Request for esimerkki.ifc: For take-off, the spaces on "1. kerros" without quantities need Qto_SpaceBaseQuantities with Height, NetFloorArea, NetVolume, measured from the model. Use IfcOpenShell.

First a look at what the model holds.

```python
import ifcopenshell
import ifcopenshell.util.element
import ifcopenshell.util.unit

model = ifcopenshell.open("esimerkki.ifc")
print(model.schema)
for unit_type in ("LENGTHUNIT", "AREAUNIT", "VOLUMEUNIT"):
    print(unit_type, ifcopenshell.util.unit.calculate_unit_scale(model, unit_type))
storey = next(s for s in model.by_type("IfcBuildingStorey") if s.Name == "1. kerros")
spaces = [e for e in ifcopenshell.util.element.get_decomposition(storey) if e.is_a("IfcSpace")]
for e in sorted(spaces, key=lambda e: e.id()):
    print(e.id(), e.is_a(), e.Name, list(ifcopenshell.util.element.get_psets(e, qtos_only=True)), sep=" | ")
```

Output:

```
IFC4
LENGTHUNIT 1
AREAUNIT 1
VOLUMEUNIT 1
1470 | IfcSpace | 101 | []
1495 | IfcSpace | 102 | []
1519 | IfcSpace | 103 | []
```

```python
import ifcopenshell
import ifcopenshell.api.pset
import ifcopenshell.geom
import ifcopenshell.util.element
import ifcopenshell.util.shape
import ifcopenshell.util.unit

model = ifcopenshell.open("esimerkki.ifc")
unit_scale = ifcopenshell.util.unit.calculate_unit_scale(model)
area_scale = ifcopenshell.util.unit.calculate_unit_scale(model, "AREAUNIT")
volume_scale = ifcopenshell.util.unit.calculate_unit_scale(model, "VOLUMEUNIT")
settings = ifcopenshell.geom.settings()

storey = next(s for s in model.by_type("IfcBuildingStorey") if s.Name == "1. kerros")
spaces = [e for e in ifcopenshell.util.element.get_decomposition(storey) if e.is_a("IfcSpace")]

for e in sorted(spaces, key=lambda e: e.id()):
    if ifcopenshell.util.element.get_psets(e, qtos_only=True, should_inherit=False):
        continue
    # Geometry comes back in metres, in the element's own axes.
    shape = ifcopenshell.geom.create_shape(settings, e)
    values = {
        "Height": ifcopenshell.util.shape.get_z(shape.geometry) / unit_scale,
        "NetFloorArea": ifcopenshell.util.shape.get_footprint_area(shape.geometry) / area_scale,
        "NetVolume": ifcopenshell.util.shape.get_volume(shape.geometry) / volume_scale,
    }
    qto = ifcopenshell.api.pset.add_qto(model, product=e, name="Qto_SpaceBaseQuantities")
    ifcopenshell.api.pset.edit_qto(model, qto=qto, properties=values)
    print(e.id(), {k: round(v, 3) for k, v in values.items()})

model.write("esimerkki_v2.ifc")
```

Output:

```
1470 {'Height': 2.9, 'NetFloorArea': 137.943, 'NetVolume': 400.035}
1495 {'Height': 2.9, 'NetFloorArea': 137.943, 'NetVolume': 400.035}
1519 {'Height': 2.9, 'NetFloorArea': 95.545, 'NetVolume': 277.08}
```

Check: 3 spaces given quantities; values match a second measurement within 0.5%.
